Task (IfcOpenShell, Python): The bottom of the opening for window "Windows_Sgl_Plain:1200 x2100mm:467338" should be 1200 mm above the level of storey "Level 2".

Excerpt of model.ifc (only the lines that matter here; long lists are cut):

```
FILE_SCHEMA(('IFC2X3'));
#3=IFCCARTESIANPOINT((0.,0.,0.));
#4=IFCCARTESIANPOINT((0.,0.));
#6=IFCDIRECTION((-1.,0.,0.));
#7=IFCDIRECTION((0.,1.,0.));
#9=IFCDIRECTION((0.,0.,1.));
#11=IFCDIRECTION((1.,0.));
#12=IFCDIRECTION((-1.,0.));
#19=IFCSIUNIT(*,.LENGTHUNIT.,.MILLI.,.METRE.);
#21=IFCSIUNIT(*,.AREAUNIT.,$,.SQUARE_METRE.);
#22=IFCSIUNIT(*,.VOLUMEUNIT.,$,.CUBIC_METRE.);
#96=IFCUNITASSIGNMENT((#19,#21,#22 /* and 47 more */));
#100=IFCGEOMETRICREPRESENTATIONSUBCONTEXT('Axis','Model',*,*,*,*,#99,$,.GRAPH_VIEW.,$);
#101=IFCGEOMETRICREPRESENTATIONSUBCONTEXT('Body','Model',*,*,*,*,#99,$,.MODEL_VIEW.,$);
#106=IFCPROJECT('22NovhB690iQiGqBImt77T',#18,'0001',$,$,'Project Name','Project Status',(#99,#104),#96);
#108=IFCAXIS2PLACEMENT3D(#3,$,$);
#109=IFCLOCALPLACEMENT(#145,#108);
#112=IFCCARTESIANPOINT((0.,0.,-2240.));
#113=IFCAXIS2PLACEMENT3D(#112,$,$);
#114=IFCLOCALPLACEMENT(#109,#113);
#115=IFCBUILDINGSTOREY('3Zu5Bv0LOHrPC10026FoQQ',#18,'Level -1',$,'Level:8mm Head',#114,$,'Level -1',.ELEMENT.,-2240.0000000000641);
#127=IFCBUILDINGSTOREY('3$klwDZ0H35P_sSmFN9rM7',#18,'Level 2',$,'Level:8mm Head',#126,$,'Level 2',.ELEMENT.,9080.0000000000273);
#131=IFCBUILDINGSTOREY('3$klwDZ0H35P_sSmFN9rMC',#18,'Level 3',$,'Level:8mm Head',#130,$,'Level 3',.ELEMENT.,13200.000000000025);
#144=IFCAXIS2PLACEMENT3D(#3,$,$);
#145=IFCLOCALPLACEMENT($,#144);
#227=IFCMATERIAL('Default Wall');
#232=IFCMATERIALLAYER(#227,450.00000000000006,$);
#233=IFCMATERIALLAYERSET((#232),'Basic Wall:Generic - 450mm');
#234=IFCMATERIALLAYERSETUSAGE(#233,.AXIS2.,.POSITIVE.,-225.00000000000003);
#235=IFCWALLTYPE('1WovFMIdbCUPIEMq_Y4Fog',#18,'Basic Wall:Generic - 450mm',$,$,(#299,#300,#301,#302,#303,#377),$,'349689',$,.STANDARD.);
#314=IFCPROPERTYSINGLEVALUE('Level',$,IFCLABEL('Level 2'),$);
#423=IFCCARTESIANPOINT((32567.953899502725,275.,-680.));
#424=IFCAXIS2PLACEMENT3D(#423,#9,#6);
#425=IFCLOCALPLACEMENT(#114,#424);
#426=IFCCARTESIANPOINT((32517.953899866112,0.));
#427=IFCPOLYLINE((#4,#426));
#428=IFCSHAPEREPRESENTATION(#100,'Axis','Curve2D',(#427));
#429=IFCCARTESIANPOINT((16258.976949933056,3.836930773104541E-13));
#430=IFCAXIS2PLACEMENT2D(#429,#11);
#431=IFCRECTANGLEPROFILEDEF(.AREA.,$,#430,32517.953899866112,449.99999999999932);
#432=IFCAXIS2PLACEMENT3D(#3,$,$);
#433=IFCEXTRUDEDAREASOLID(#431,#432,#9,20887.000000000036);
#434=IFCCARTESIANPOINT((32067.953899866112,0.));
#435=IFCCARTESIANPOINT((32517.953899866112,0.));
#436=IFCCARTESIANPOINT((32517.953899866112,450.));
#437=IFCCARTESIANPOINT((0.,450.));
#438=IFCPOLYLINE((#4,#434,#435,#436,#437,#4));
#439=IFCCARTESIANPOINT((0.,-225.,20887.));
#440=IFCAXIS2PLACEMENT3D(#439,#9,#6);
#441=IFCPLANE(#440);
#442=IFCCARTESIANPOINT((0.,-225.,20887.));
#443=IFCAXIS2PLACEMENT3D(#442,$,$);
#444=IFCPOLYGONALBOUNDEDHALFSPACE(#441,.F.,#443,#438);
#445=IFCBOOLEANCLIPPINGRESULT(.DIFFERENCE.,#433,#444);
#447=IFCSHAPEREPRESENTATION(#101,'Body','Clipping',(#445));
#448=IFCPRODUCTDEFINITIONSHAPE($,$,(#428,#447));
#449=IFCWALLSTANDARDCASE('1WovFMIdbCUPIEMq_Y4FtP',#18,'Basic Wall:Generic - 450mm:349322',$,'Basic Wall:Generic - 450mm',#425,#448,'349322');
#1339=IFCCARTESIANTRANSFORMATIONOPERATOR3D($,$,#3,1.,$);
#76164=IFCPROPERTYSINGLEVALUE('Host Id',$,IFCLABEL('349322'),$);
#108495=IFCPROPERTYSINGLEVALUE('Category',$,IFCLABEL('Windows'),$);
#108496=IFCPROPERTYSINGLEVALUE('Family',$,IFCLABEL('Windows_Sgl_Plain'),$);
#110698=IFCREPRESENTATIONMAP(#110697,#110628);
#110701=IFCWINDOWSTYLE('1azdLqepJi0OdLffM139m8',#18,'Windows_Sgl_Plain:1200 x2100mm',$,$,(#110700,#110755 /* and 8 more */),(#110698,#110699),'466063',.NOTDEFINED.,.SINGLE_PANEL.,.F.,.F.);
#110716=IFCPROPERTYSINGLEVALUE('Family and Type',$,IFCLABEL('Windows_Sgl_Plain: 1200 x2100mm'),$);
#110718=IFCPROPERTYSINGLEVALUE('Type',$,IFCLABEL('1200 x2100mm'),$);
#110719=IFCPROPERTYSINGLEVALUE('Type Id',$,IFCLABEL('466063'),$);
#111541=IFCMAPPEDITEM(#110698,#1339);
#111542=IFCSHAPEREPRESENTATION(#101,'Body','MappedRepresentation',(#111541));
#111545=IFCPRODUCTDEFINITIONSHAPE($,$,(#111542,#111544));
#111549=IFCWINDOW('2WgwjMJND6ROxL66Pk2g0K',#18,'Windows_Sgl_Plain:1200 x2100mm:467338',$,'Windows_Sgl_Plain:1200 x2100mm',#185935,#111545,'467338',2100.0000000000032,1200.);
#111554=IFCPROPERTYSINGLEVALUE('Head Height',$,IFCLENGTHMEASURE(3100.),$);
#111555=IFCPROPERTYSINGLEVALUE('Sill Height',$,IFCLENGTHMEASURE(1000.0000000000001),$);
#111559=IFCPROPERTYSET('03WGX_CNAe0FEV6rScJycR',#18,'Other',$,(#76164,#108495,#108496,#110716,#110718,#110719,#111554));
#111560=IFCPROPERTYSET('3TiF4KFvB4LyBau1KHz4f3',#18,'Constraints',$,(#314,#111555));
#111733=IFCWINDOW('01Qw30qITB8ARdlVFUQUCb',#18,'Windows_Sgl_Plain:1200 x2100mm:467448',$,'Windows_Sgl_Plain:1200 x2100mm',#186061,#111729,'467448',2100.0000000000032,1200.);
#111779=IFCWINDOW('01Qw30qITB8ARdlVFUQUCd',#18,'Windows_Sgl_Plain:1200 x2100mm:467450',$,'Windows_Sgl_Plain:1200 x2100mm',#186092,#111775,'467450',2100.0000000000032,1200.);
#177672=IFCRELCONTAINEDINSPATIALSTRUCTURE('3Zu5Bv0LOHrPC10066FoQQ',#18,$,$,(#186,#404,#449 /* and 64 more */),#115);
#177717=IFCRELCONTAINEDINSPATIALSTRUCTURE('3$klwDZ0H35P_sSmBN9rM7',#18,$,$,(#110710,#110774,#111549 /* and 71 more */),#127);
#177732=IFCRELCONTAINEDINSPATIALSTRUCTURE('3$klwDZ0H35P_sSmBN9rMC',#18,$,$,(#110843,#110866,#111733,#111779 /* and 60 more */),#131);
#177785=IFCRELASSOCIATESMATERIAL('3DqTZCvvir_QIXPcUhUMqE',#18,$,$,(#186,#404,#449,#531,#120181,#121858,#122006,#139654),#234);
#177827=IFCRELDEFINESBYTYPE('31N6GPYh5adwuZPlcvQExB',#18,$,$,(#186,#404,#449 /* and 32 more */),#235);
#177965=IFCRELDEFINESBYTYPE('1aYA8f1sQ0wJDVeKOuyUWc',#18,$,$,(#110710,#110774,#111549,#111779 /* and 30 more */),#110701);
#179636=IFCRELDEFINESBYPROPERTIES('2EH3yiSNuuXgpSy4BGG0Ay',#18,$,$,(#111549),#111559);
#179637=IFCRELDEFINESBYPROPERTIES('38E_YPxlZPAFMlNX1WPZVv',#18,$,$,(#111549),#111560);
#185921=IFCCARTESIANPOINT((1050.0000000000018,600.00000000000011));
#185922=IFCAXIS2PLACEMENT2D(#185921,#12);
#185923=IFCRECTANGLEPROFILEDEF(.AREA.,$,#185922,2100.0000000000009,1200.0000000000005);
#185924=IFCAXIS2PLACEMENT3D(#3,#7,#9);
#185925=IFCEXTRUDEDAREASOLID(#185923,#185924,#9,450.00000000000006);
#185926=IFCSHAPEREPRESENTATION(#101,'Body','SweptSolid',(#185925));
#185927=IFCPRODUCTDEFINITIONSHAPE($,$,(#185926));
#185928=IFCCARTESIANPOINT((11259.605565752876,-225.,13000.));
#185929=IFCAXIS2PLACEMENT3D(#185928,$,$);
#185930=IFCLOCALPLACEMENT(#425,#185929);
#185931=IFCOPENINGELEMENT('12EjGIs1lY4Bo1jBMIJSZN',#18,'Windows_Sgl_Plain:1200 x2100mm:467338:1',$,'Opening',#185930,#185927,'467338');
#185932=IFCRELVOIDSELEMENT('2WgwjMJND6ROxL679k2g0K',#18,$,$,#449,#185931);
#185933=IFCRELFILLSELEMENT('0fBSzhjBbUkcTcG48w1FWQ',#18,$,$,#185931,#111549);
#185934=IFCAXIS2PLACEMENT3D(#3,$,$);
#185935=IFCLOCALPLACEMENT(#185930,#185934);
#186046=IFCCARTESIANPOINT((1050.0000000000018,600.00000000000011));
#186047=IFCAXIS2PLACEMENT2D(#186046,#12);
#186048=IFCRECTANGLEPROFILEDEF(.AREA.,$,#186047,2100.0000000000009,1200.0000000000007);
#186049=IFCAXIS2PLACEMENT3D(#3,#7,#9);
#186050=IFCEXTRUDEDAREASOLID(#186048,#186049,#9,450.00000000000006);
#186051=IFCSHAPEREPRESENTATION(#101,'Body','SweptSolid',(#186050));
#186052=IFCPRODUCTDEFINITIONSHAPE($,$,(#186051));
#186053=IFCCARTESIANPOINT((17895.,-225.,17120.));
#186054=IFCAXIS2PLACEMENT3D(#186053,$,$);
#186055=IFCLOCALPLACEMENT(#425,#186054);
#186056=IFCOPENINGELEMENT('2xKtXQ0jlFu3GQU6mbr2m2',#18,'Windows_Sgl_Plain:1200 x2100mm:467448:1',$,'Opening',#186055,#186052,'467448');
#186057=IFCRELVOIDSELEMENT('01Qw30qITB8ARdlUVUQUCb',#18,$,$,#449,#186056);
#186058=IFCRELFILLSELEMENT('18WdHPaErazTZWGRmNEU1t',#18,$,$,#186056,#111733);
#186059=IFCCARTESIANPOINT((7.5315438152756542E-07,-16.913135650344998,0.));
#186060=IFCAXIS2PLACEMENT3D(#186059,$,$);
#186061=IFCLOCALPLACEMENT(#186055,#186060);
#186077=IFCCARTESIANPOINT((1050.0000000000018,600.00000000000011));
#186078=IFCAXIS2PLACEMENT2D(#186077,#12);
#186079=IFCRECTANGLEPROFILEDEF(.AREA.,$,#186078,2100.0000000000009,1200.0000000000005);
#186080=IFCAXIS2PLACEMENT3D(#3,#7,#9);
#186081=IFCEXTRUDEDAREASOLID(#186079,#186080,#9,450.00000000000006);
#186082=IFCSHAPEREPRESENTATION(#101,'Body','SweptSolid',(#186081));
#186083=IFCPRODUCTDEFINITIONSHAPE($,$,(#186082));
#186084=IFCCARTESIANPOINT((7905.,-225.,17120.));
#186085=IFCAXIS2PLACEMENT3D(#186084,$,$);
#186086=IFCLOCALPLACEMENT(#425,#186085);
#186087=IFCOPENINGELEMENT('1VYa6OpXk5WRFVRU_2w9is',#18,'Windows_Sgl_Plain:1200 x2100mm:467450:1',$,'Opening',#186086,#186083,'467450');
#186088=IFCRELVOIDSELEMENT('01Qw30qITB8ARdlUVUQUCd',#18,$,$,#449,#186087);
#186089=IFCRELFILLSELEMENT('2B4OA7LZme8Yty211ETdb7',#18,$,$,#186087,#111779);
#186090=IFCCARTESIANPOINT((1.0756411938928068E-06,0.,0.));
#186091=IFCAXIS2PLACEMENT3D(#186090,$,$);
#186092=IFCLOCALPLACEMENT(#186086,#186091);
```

```python
import numpy as np
import ifcopenshell
import ifcopenshell.api.geometry
import ifcopenshell.api.pset
import ifcopenshell.geom
import ifcopenshell.util.element
import ifcopenshell.util.placement
import ifcopenshell.util.shape
import ifcopenshell.util.unit

model = ifcopenshell.open("model.ifc")
unit_scale = ifcopenshell.util.unit.calculate_unit_scale(model)

window = model.by_guid("2WgwjMJND6ROxL66Pk2g0K")
opening = window.FillsVoids[0].RelatingOpeningElement
storey = ifcopenshell.util.element.get_container(window, ifc_class="IfcBuildingStorey")
level = ifcopenshell.util.placement.get_local_placement(storey.ObjectPlacement)[2, 3]

# The opening's origin need not be at the sill, so measure its lowest point.
shape = ifcopenshell.geom.create_shape(ifcopenshell.geom.settings(), opening)
bottom = ifcopenshell.util.shape.get_shape_bottom_elevation(shape, shape.geometry) / unit_scale
dz = level + 1200.0 - bottom

shift = np.array([0.0, 0.0, dz])
# The window is placed relative to its opening, so it follows when the opening moves.
matrix = ifcopenshell.util.placement.get_local_placement(opening.ObjectPlacement)
matrix[:3, 3] += shift
ifcopenshell.api.geometry.edit_object_placement(
    model, product=opening, matrix=matrix, is_si=False, should_transform_children=True
)

# Keep the stored heights in step.
pset = model.by_id(ifcopenshell.util.element.get_pset(window, "Other", should_inherit=False)["id"])
ifcopenshell.api.pset.edit_pset(model, pset=pset, properties={
    "Head Height": model.create_entity("IfcLengthMeasure", ifcopenshell.util.element.get_pset(window, "Other", "Head Height") + dz),
})
pset = model.by_id(ifcopenshell.util.element.get_pset(window, "Constraints", should_inherit=False)["id"])
ifcopenshell.api.pset.edit_pset(model, pset=pset, properties={
    "Sill Height": model.create_entity("IfcLengthMeasure", ifcopenshell.util.element.get_pset(window, "Constraints", "Sill Height") + dz),
})

print(f"moved by {dz * unit_scale:+.3f} m")

model.write("model_rev.ifc")
```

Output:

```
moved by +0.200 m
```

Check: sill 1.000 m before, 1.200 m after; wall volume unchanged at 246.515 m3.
